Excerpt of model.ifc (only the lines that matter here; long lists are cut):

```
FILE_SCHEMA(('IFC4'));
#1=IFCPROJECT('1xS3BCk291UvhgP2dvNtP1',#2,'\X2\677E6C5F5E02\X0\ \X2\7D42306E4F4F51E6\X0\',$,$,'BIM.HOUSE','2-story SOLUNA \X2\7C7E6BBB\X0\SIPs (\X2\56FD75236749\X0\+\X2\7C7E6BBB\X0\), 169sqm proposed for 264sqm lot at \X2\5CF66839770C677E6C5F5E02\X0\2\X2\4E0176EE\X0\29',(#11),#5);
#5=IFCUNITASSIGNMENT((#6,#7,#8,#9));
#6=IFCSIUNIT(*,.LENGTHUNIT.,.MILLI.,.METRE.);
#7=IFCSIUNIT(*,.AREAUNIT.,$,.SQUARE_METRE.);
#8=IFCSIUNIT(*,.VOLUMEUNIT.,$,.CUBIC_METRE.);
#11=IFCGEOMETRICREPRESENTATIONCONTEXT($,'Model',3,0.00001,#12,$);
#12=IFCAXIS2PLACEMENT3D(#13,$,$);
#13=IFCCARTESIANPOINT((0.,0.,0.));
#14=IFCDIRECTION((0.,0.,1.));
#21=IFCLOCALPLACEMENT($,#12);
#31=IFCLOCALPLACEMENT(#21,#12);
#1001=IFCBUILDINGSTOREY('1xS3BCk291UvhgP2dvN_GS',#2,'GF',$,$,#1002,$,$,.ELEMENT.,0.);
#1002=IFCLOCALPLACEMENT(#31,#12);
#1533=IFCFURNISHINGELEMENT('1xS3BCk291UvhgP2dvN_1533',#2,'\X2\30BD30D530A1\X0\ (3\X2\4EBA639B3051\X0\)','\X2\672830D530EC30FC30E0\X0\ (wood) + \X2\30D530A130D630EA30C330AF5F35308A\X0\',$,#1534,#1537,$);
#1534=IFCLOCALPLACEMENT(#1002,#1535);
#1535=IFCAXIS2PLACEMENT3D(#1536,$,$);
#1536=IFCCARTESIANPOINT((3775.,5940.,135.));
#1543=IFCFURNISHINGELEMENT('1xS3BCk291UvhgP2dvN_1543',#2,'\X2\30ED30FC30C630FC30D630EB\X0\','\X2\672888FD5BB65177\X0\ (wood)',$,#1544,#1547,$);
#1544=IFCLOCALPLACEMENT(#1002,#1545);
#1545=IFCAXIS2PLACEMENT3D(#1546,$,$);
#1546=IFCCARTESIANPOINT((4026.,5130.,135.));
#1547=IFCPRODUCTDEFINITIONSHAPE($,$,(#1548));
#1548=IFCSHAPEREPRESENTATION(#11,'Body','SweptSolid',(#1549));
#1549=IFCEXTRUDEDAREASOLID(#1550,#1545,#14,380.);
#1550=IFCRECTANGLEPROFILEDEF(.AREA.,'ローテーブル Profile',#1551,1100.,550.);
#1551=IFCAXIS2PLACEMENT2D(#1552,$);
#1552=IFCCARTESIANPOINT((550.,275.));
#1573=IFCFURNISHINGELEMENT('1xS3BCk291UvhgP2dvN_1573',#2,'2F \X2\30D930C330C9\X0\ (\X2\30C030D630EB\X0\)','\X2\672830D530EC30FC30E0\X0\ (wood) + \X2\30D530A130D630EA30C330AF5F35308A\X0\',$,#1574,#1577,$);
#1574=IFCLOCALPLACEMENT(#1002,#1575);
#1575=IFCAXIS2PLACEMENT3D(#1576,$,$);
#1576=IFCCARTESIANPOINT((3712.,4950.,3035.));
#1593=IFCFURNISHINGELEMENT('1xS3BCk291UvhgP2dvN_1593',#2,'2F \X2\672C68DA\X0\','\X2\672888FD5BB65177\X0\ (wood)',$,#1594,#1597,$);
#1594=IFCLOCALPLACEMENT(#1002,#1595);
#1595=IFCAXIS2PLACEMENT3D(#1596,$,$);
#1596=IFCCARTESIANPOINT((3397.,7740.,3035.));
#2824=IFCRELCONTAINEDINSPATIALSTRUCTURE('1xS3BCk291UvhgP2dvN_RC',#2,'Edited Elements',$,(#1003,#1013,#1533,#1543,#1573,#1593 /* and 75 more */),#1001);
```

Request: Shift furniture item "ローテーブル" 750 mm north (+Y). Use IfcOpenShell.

```python
import ifcopenshell
import ifcopenshell.api.geometry
import ifcopenshell.util.placement
import ifcopenshell.util.unit

model = ifcopenshell.open("model.ifc")
unit_scale = ifcopenshell.util.unit.calculate_unit_scale(model)

item = model.by_guid("1xS3BCk291UvhgP2dvN_1543")
matrix = ifcopenshell.util.placement.get_local_placement(item.ObjectPlacement)
matrix[1, 3] += 0.75 / unit_scale
ifcopenshell.api.geometry.edit_object_placement(model, product=item, matrix=matrix, is_si=False)

print(ifcopenshell.util.placement.get_local_placement(item.ObjectPlacement).round(3) + 0.0)

model.write("model_v2.ifc")
```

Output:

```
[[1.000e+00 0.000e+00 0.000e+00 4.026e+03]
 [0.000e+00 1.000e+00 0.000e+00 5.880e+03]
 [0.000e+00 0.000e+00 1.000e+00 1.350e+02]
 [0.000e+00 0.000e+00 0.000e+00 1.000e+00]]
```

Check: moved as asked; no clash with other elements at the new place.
